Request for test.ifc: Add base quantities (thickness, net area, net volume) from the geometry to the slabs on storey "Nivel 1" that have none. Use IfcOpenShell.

First a look at what the model holds.

```python
import ifcopenshell
import ifcopenshell.util.element
import ifcopenshell.util.unit

model = ifcopenshell.open("test.ifc")
print(model.schema)
for unit_type in ("LENGTHUNIT", "AREAUNIT", "VOLUMEUNIT"):
    print(unit_type, ifcopenshell.util.unit.calculate_unit_scale(model, unit_type))
storey = next(s for s in model.by_type("IfcBuildingStorey") if s.Name == "Nivel 1")
slabs = [e for e in ifcopenshell.util.element.get_decomposition(storey) if e.is_a("IfcSlab")]
for e in sorted(slabs, key=lambda e: e.id()):
    print(e.id(), e.is_a(), e.Name, list(ifcopenshell.util.element.get_psets(e, qtos_only=True)), sep=" | ")
```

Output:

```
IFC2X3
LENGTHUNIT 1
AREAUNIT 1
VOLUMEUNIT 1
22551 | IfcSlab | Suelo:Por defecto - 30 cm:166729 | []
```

```python
import ifcopenshell
import ifcopenshell.api.pset
import ifcopenshell.geom
import ifcopenshell.util.element
import ifcopenshell.util.shape
import ifcopenshell.util.unit

model = ifcopenshell.open("test.ifc")
unit_scale = ifcopenshell.util.unit.calculate_unit_scale(model)
area_scale = ifcopenshell.util.unit.calculate_unit_scale(model, "AREAUNIT")
volume_scale = ifcopenshell.util.unit.calculate_unit_scale(model, "VOLUMEUNIT")
settings = ifcopenshell.geom.settings()

storey = next(s for s in model.by_type("IfcBuildingStorey") if s.Name == "Nivel 1")
slabs = [e for e in ifcopenshell.util.element.get_decomposition(storey) if e.is_a("IfcSlab")]

for e in sorted(slabs, key=lambda e: e.id()):
    if ifcopenshell.util.element.get_psets(e, qtos_only=True, should_inherit=False):
        continue
    # Geometry comes back in metres, in the element's own axes.
    shape = ifcopenshell.geom.create_shape(settings, e)
    values = {
        "Width": ifcopenshell.util.shape.get_z(shape.geometry) / unit_scale,
        "NetArea": ifcopenshell.util.shape.get_footprint_area(shape.geometry) / area_scale,
        "NetVolume": ifcopenshell.util.shape.get_volume(shape.geometry) / volume_scale,
    }
    qto = ifcopenshell.api.pset.add_qto(model, product=e, name="BaseQuantities")
    ifcopenshell.api.pset.edit_qto(model, qto=qto, properties=values)
    print(e.id(), {k: round(v, 3) for k, v in values.items()})

model.write("test_rev.ifc")
```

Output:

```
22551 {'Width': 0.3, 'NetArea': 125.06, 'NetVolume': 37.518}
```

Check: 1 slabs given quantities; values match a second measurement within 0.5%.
